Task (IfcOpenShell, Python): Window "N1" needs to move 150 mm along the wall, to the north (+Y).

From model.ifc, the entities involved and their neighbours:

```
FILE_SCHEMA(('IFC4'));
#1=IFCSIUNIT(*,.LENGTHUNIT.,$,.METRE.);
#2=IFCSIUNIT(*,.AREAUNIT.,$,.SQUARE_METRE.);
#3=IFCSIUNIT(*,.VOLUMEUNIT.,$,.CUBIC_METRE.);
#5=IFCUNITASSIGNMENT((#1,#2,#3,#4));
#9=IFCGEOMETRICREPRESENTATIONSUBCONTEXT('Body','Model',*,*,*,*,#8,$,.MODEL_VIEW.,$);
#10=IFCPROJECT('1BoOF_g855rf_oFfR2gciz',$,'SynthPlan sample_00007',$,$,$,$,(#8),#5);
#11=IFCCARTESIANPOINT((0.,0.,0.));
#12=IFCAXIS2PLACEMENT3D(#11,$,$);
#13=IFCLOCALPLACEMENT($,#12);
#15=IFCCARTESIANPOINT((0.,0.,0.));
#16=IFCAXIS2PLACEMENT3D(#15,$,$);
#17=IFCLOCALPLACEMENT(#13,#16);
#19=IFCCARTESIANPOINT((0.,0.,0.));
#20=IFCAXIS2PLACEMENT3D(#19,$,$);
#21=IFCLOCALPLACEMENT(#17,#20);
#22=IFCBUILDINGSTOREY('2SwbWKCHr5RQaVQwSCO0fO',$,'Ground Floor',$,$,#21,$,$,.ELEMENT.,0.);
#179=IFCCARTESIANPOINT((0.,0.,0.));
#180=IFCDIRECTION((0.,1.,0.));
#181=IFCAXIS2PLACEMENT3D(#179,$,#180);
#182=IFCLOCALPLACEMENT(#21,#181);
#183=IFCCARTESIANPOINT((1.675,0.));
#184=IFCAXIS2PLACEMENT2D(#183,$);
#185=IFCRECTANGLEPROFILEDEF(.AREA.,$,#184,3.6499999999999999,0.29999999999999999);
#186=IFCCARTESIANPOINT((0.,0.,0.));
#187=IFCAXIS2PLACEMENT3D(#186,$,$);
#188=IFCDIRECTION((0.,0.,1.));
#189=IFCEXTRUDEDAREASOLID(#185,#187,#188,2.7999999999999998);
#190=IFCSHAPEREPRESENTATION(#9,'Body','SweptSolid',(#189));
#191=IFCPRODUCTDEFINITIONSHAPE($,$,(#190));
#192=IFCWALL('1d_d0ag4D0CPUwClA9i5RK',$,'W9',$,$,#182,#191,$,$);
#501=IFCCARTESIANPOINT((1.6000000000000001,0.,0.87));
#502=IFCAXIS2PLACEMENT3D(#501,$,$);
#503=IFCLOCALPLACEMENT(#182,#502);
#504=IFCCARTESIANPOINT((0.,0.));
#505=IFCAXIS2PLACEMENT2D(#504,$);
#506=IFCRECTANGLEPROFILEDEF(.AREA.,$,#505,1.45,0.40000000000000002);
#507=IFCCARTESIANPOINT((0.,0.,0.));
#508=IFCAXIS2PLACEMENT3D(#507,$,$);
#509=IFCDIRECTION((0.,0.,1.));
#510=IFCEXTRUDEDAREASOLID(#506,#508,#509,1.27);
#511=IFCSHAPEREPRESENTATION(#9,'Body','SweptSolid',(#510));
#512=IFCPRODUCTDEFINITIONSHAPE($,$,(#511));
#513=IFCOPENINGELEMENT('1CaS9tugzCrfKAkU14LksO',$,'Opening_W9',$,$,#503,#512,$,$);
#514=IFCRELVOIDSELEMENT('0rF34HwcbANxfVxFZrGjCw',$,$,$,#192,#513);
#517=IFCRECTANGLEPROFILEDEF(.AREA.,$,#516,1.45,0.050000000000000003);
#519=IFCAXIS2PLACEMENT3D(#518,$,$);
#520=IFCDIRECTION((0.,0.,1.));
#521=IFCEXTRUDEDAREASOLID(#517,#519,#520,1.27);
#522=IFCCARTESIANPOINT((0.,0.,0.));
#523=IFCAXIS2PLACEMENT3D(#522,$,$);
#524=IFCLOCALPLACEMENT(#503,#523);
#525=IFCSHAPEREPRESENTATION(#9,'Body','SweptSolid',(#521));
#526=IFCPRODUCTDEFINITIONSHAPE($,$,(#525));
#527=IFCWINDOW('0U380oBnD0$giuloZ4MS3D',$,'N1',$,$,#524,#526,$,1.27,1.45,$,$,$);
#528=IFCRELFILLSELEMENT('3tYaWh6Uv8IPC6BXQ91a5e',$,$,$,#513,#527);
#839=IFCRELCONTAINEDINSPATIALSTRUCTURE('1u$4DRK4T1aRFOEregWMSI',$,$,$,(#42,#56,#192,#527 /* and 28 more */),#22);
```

```python
import ifcopenshell
import ifcopenshell.api.geometry
import ifcopenshell.util.placement
import ifcopenshell.util.unit

model = ifcopenshell.open("model.ifc")
unit_scale = ifcopenshell.util.unit.calculate_unit_scale(model)

window = model.by_guid("0U380oBnD0$giuloZ4MS3D")
opening = window.FillsVoids[0].RelatingOpeningElement
wall = opening.VoidsElements[0].RelatingBuildingElement

wall_matrix = ifcopenshell.util.placement.get_local_placement(wall.ObjectPlacement)
shift = wall_matrix[:3, 0] * 0.15 / unit_scale
before = ifcopenshell.util.placement.get_local_placement(window.ObjectPlacement)[:3, 3].copy()

# The window is placed relative to its opening, so it follows when the opening moves.
matrix = ifcopenshell.util.placement.get_local_placement(opening.ObjectPlacement)
matrix[:3, 3] += shift
ifcopenshell.api.geometry.edit_object_placement(
    model, product=opening, matrix=matrix, is_si=False, should_transform_children=True
)

after = ifcopenshell.util.placement.get_local_placement(window.ObjectPlacement)[:3, 3]
print("window moved by", (after - before).round(3) + 0.0)

model.write("model_v2.ifc")
```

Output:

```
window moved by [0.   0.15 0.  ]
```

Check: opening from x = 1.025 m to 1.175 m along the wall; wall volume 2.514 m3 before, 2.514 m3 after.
